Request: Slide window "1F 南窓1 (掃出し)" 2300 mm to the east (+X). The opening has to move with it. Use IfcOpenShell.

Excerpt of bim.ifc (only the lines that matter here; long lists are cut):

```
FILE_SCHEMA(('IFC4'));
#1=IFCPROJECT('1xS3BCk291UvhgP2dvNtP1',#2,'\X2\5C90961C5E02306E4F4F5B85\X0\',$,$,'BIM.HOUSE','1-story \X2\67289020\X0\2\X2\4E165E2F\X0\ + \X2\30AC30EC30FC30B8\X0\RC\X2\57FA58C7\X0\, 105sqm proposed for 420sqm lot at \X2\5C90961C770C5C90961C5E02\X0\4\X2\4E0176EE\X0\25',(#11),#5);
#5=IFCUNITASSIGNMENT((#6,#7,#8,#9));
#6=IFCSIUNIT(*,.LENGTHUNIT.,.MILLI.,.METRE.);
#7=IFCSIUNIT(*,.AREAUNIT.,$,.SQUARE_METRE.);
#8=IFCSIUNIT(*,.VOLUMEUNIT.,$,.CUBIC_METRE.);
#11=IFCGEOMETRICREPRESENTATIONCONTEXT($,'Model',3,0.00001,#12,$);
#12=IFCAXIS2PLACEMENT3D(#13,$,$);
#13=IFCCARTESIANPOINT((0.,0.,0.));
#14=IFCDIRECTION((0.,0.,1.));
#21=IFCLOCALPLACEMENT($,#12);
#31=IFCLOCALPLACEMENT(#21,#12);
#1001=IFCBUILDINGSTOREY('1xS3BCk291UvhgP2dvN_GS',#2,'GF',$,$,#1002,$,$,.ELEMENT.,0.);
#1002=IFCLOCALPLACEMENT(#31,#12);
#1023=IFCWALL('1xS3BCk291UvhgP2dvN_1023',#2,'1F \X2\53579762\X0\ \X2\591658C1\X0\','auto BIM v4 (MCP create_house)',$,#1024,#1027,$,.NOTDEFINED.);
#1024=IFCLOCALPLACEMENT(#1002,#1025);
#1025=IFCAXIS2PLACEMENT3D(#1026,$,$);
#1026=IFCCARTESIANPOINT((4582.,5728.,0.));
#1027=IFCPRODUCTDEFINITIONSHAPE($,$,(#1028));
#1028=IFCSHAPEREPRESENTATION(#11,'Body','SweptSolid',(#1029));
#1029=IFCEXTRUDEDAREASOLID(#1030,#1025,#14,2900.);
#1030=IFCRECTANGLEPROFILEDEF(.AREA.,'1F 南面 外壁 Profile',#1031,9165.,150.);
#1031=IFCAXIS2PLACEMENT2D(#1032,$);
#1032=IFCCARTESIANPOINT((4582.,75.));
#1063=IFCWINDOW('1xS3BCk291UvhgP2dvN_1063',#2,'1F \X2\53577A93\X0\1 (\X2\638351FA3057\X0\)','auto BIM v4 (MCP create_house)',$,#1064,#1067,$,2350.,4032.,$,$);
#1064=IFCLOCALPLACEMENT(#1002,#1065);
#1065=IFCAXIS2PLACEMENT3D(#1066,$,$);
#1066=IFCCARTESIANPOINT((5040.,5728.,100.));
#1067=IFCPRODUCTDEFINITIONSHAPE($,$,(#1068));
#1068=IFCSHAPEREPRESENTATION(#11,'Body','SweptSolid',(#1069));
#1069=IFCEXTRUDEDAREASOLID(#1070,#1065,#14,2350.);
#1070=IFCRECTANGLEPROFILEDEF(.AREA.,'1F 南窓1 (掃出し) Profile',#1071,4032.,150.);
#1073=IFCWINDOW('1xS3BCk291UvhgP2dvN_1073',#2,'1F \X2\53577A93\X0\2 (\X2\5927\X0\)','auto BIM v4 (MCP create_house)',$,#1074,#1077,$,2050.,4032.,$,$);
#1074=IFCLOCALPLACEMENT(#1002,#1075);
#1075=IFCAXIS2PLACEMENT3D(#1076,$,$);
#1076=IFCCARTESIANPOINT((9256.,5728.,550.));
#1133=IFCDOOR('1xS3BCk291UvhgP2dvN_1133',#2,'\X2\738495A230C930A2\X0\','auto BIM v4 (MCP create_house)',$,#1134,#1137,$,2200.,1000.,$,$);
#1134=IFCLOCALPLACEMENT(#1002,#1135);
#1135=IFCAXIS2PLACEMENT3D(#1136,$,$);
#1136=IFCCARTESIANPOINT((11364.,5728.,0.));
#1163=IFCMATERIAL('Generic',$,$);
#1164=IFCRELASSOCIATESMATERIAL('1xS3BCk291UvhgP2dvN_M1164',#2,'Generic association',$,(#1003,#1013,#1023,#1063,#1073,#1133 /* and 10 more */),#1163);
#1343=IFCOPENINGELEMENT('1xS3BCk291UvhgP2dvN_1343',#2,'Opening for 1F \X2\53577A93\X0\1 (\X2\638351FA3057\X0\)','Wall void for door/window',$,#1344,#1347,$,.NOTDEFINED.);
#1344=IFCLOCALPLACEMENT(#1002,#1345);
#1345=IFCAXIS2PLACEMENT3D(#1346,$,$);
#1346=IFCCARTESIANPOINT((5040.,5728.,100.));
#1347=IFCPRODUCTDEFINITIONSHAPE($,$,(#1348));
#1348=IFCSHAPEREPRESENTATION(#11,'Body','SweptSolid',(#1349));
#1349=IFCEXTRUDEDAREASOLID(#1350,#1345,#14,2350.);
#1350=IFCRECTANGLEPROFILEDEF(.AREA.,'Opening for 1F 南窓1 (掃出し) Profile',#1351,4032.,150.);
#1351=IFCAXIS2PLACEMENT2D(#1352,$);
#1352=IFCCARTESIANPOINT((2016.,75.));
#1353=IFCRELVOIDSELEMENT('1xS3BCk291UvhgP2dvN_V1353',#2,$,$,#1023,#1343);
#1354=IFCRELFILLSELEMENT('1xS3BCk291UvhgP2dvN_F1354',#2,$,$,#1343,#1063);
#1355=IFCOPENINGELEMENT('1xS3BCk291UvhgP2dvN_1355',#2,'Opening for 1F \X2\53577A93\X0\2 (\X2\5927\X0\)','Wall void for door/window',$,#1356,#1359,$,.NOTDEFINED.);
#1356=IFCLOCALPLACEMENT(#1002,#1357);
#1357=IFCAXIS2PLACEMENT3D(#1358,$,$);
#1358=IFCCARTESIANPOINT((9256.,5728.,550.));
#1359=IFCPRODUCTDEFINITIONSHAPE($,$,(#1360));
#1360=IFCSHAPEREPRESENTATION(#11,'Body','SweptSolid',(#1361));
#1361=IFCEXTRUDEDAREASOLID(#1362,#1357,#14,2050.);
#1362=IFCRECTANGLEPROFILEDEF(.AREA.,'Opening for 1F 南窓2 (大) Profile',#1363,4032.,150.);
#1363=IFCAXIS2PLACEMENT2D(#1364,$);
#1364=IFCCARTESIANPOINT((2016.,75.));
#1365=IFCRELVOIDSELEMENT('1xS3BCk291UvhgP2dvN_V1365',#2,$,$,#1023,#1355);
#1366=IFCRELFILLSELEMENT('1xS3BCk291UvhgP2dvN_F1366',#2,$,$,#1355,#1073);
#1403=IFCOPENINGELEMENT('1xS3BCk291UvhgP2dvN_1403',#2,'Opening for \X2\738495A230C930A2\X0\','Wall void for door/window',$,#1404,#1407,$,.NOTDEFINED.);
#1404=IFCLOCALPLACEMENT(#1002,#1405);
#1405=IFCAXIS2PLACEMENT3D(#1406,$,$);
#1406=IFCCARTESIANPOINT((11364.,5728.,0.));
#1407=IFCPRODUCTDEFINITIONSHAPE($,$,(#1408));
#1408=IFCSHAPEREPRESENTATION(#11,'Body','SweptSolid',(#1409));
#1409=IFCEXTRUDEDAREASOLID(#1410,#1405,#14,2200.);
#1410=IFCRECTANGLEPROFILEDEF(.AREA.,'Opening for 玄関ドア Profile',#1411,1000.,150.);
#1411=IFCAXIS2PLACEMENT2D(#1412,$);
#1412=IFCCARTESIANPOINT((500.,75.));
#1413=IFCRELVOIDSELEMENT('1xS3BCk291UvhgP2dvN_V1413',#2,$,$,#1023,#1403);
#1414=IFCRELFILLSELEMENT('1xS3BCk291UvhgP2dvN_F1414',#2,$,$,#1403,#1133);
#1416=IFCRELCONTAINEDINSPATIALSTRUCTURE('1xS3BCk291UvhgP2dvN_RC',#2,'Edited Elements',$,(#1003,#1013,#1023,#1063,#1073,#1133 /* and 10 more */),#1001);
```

```python
import ifcopenshell
import ifcopenshell.api.geometry
import ifcopenshell.util.placement

model = ifcopenshell.open("bim.ifc")

window = model.by_guid("1xS3BCk291UvhgP2dvN_1063")
opening = window.FillsVoids[0].RelatingOpeningElement
wall = opening.VoidsElements[0].RelatingBuildingElement

wall_matrix = ifcopenshell.util.placement.get_local_placement(wall.ObjectPlacement)
shift = wall_matrix[:3, 0] * 2300.0
before = ifcopenshell.util.placement.get_local_placement(window.ObjectPlacement)[:3, 3].copy()

# The window is not placed relative to its opening, so move both.
for product in (opening, window):
    matrix = ifcopenshell.util.placement.get_local_placement(product.ObjectPlacement)
    matrix[:3, 3] += shift
    ifcopenshell.api.geometry.edit_object_placement(model, product=product, matrix=matrix, is_si=False)

after = ifcopenshell.util.placement.get_local_placement(window.ObjectPlacement)[:3, 3]
print("window moved by", (after - before).round(3) + 0.0)

model.write("bim_edited.ifc")
```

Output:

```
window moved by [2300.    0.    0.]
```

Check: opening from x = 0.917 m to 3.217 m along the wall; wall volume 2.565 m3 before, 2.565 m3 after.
